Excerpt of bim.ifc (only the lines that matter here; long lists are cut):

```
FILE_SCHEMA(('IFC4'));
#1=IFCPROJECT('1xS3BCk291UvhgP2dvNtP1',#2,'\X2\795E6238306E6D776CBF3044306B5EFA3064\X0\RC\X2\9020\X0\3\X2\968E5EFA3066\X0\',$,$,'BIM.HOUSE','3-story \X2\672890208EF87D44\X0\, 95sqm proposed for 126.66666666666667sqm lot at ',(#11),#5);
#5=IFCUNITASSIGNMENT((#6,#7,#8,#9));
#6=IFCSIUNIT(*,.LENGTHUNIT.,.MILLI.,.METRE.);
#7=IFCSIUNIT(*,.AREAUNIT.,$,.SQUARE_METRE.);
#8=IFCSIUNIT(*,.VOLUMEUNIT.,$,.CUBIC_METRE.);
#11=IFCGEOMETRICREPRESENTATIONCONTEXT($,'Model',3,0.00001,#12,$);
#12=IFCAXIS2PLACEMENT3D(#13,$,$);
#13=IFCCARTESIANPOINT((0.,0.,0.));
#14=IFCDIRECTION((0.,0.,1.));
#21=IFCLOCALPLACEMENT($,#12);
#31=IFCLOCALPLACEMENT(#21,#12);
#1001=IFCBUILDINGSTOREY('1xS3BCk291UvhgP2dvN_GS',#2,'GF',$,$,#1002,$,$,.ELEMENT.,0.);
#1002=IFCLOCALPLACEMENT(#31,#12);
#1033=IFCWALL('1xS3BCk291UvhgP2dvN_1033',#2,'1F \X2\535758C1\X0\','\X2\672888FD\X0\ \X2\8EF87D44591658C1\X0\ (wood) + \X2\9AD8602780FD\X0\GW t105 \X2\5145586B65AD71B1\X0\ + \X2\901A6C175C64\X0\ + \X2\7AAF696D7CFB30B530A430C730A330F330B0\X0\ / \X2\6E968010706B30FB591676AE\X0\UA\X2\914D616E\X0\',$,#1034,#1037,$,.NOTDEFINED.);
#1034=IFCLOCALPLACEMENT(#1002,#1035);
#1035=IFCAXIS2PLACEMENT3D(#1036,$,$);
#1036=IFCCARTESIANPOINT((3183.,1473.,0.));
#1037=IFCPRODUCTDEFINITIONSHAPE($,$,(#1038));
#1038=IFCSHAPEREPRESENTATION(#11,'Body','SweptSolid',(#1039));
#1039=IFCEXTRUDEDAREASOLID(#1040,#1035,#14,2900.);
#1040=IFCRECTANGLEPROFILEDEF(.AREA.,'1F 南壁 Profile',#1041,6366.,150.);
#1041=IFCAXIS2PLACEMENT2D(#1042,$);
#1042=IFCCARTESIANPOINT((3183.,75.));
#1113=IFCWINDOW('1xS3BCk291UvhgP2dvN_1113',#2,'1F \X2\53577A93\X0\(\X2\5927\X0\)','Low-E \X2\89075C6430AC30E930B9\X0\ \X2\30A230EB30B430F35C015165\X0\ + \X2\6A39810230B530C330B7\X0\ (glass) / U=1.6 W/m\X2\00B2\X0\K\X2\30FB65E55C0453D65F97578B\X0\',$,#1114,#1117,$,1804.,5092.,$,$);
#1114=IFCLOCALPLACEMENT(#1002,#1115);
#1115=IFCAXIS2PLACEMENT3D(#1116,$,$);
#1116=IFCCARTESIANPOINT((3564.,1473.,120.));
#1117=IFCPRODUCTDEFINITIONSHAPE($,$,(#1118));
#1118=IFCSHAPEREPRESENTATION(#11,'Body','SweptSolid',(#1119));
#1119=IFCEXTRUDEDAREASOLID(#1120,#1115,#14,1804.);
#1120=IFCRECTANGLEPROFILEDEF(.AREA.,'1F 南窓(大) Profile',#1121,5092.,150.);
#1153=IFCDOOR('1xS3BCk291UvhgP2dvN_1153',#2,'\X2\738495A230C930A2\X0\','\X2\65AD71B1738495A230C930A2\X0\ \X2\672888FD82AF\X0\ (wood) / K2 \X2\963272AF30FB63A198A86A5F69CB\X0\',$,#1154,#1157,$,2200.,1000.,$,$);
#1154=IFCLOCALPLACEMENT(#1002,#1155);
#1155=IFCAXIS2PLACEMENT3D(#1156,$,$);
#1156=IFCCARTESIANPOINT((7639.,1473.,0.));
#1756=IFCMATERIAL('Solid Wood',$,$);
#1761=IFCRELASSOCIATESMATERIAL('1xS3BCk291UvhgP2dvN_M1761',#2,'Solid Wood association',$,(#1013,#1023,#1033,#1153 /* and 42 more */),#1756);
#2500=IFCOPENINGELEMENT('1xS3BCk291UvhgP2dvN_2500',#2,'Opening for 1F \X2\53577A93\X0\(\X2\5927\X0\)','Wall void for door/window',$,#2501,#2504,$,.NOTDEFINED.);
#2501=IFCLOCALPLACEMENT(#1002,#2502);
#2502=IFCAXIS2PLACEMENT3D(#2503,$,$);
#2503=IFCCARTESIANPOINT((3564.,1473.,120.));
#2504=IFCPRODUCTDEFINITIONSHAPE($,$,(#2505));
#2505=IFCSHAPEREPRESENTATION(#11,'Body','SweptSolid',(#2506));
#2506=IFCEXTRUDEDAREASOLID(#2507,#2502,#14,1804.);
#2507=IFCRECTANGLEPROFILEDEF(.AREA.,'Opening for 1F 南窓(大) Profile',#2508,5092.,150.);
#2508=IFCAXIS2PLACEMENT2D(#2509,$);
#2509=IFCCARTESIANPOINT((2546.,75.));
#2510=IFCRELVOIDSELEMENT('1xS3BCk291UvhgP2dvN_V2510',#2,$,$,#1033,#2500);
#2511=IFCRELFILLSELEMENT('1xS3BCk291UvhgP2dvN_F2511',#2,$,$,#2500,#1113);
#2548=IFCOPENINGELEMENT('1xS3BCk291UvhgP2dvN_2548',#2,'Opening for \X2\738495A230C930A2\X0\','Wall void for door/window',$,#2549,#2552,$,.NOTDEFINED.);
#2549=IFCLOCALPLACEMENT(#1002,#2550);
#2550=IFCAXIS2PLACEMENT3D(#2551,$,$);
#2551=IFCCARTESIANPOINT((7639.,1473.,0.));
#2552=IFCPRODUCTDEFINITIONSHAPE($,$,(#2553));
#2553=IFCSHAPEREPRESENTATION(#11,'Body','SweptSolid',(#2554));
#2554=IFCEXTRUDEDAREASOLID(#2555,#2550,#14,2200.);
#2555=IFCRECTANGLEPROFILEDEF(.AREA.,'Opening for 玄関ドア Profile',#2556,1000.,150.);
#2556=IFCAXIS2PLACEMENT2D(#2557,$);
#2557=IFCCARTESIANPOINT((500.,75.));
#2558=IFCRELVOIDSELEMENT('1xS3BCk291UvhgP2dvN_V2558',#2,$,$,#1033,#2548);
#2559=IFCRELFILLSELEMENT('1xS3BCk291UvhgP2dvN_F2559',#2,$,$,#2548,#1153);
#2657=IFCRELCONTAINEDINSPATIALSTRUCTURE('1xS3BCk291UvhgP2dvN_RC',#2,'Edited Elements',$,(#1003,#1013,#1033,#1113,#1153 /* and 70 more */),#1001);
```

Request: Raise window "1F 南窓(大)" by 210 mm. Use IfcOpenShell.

```python
import numpy as np
import ifcopenshell
import ifcopenshell.api.geometry
import ifcopenshell.util.placement
import ifcopenshell.util.unit

model = ifcopenshell.open("bim.ifc")
unit_scale = ifcopenshell.util.unit.calculate_unit_scale(model)

window = model.by_guid("1xS3BCk291UvhgP2dvN_1113")
opening = window.FillsVoids[0].RelatingOpeningElement
dz = 0.21 / unit_scale

shift = np.array([0.0, 0.0, dz])
# The window is not placed relative to its opening, so move both.
for product in (opening, window):
    matrix = ifcopenshell.util.placement.get_local_placement(product.ObjectPlacement)
    matrix[:3, 3] += shift
    ifcopenshell.api.geometry.edit_object_placement(model, product=product, matrix=matrix, is_si=False)

print(f"moved by {dz * unit_scale:+.3f} m")

model.write("bim_v2.ifc")
```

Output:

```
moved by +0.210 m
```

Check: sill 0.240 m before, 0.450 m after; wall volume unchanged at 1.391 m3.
